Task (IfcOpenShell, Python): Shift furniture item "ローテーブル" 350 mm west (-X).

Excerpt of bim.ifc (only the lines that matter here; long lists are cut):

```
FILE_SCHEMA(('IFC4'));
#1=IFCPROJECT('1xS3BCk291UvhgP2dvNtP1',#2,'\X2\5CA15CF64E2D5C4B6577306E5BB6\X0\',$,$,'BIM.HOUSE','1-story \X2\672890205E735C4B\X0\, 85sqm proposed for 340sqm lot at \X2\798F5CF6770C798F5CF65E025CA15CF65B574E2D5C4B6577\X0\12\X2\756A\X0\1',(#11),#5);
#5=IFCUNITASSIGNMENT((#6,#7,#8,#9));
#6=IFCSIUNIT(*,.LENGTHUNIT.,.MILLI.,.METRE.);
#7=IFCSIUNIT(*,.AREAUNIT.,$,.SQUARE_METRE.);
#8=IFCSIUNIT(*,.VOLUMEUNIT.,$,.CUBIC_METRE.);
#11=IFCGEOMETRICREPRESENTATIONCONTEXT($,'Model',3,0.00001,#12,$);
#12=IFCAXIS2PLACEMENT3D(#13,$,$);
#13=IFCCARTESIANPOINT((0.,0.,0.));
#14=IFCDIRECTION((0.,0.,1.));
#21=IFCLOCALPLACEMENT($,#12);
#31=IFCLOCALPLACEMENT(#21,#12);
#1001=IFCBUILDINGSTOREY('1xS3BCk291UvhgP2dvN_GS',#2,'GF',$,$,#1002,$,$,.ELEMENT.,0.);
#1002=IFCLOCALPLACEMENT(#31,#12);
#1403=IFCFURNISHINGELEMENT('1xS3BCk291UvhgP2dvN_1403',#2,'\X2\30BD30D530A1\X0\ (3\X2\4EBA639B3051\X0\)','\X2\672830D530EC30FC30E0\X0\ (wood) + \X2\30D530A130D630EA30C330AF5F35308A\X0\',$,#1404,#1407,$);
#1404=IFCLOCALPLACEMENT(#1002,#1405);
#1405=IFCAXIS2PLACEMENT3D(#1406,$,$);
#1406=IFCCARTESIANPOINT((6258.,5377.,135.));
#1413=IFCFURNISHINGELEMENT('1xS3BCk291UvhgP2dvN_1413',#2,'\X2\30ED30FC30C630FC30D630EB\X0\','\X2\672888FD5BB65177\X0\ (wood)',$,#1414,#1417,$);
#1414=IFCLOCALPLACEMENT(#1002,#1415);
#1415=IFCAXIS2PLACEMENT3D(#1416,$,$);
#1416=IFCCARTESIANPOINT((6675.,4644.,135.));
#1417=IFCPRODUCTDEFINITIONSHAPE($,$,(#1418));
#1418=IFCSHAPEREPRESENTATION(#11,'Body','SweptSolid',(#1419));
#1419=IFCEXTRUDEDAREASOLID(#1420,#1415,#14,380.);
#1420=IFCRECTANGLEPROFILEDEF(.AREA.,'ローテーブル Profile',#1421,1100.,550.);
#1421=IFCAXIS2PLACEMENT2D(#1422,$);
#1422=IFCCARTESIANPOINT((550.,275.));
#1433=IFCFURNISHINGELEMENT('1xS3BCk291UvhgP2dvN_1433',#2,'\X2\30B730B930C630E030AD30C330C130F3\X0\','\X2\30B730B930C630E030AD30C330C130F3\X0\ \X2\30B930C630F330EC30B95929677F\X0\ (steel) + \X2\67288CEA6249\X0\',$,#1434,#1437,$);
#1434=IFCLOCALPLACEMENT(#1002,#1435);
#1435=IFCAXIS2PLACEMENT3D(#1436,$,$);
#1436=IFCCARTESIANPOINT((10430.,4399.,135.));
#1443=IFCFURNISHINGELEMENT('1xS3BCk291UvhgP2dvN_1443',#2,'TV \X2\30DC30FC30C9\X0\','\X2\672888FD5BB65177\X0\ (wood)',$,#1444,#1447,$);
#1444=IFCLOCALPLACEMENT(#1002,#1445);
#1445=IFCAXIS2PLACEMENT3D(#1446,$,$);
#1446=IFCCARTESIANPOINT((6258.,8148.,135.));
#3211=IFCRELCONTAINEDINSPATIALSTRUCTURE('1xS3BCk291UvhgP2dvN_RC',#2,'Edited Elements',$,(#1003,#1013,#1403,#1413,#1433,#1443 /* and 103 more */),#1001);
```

```python
import ifcopenshell
import ifcopenshell.api.geometry
import ifcopenshell.util.placement
import ifcopenshell.util.unit

model = ifcopenshell.open("bim.ifc")
unit_scale = ifcopenshell.util.unit.calculate_unit_scale(model)

item = model.by_id(1413)
matrix = ifcopenshell.util.placement.get_local_placement(item.ObjectPlacement)
matrix[0, 3] -= 0.35 / unit_scale
ifcopenshell.api.geometry.edit_object_placement(model, product=item, matrix=matrix, is_si=False)

print(ifcopenshell.util.placement.get_local_placement(item.ObjectPlacement).round(3) + 0.0)

model.write("bim_rev.ifc")
```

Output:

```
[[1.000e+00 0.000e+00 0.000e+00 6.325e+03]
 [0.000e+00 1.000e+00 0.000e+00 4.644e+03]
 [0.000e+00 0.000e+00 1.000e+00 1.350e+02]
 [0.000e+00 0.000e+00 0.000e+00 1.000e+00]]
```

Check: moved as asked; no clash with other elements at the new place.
